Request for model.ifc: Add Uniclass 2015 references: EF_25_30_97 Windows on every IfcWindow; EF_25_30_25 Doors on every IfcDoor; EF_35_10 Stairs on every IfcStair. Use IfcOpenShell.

First a look at what the model holds.

```python
import ifcopenshell

model = ifcopenshell.open("model.ifc")
print(model.schema)
print("classifications:", [c.Name for c in model.by_type("IfcClassification")])
for ifc_class in ("IfcDoor", "IfcRoof", "IfcStair", "IfcWall", "IfcWindow"):
    print(ifc_class, len(model.by_type(ifc_class)))
```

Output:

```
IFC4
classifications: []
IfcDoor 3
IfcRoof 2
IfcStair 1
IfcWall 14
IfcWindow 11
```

```python
import ifcopenshell
import ifcopenshell.api.classification

model = ifcopenshell.open("model.ifc")

system = ifcopenshell.api.classification.add_classification(model, classification="Uniclass 2015")

codes = {
    "IfcWindow": ("EF_25_30_97", "Windows"),
    "IfcDoor": ("EF_25_30_25", "Doors"),
    "IfcStair": ("EF_35_10", "Stairs"),
}
for ifc_class, (code, name) in codes.items():
    products = model.by_type(ifc_class)
    ifcopenshell.api.classification.add_reference(
        model, products=products, classification=system, identification=code, name=name
    )
    print(code, len(products))

model.write("model_v2.ifc")
```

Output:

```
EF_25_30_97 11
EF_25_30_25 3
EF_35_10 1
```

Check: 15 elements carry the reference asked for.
